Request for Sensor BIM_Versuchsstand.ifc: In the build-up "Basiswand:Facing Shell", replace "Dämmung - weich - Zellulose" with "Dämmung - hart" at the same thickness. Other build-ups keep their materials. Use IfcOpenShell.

First a look at what the model holds.

```python
import ifcopenshell
import ifcopenshell.util.element

model = ifcopenshell.open("Sensor BIM_Versuchsstand.ifc")
print(model.schema)
for layer_set in model.by_type("IfcMaterialLayerSet"):
    if layer_set.LayerSetName == "Basiswand:Facing Shell":
        for layer in layer_set.MaterialLayers:
            print(layer.id(), layer.Material and layer.Material.Name, layer.LayerThickness, sep=" | ")
        print(len(ifcopenshell.util.element.get_elements_by_material(model, layer_set)), "elements and types use it")
print(sorted(m.Name for m in model.by_type("IfcMaterial") if m.Name)[:60])
```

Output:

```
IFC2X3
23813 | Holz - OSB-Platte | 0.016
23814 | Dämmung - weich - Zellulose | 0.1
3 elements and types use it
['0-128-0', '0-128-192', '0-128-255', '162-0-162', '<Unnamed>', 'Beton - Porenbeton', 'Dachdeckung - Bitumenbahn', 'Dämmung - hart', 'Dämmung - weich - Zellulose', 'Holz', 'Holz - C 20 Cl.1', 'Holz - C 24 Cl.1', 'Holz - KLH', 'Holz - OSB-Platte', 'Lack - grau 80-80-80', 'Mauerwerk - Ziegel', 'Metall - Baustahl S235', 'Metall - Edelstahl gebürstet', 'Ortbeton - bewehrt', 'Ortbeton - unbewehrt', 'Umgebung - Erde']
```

```python
import ifcopenshell
import ifcopenshell.api.material

model = ifcopenshell.open("Sensor BIM_Versuchsstand.ifc")

layer_set = next(s for s in model.by_type("IfcMaterialLayerSet") if s.LayerSetName == "Basiswand:Facing Shell")
layer = next(l for l in layer_set.MaterialLayers if l.Material and l.Material.Name == "Dämmung - weich - Zellulose")
material = next(m for m in model.by_type("IfcMaterial") if m.Name == "Dämmung - hart")

# Point this one layer at the other material; renaming the old one would change it everywhere.
ifcopenshell.api.material.edit_layer(model, layer=layer, attributes={}, material=material)

print([l.Material.Name if l.Material else None for l in layer_set.MaterialLayers])

model.write("Sensor BIM_Versuchsstand_updated.ifc")
```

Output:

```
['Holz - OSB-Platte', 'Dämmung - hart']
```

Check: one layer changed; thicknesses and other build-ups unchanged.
